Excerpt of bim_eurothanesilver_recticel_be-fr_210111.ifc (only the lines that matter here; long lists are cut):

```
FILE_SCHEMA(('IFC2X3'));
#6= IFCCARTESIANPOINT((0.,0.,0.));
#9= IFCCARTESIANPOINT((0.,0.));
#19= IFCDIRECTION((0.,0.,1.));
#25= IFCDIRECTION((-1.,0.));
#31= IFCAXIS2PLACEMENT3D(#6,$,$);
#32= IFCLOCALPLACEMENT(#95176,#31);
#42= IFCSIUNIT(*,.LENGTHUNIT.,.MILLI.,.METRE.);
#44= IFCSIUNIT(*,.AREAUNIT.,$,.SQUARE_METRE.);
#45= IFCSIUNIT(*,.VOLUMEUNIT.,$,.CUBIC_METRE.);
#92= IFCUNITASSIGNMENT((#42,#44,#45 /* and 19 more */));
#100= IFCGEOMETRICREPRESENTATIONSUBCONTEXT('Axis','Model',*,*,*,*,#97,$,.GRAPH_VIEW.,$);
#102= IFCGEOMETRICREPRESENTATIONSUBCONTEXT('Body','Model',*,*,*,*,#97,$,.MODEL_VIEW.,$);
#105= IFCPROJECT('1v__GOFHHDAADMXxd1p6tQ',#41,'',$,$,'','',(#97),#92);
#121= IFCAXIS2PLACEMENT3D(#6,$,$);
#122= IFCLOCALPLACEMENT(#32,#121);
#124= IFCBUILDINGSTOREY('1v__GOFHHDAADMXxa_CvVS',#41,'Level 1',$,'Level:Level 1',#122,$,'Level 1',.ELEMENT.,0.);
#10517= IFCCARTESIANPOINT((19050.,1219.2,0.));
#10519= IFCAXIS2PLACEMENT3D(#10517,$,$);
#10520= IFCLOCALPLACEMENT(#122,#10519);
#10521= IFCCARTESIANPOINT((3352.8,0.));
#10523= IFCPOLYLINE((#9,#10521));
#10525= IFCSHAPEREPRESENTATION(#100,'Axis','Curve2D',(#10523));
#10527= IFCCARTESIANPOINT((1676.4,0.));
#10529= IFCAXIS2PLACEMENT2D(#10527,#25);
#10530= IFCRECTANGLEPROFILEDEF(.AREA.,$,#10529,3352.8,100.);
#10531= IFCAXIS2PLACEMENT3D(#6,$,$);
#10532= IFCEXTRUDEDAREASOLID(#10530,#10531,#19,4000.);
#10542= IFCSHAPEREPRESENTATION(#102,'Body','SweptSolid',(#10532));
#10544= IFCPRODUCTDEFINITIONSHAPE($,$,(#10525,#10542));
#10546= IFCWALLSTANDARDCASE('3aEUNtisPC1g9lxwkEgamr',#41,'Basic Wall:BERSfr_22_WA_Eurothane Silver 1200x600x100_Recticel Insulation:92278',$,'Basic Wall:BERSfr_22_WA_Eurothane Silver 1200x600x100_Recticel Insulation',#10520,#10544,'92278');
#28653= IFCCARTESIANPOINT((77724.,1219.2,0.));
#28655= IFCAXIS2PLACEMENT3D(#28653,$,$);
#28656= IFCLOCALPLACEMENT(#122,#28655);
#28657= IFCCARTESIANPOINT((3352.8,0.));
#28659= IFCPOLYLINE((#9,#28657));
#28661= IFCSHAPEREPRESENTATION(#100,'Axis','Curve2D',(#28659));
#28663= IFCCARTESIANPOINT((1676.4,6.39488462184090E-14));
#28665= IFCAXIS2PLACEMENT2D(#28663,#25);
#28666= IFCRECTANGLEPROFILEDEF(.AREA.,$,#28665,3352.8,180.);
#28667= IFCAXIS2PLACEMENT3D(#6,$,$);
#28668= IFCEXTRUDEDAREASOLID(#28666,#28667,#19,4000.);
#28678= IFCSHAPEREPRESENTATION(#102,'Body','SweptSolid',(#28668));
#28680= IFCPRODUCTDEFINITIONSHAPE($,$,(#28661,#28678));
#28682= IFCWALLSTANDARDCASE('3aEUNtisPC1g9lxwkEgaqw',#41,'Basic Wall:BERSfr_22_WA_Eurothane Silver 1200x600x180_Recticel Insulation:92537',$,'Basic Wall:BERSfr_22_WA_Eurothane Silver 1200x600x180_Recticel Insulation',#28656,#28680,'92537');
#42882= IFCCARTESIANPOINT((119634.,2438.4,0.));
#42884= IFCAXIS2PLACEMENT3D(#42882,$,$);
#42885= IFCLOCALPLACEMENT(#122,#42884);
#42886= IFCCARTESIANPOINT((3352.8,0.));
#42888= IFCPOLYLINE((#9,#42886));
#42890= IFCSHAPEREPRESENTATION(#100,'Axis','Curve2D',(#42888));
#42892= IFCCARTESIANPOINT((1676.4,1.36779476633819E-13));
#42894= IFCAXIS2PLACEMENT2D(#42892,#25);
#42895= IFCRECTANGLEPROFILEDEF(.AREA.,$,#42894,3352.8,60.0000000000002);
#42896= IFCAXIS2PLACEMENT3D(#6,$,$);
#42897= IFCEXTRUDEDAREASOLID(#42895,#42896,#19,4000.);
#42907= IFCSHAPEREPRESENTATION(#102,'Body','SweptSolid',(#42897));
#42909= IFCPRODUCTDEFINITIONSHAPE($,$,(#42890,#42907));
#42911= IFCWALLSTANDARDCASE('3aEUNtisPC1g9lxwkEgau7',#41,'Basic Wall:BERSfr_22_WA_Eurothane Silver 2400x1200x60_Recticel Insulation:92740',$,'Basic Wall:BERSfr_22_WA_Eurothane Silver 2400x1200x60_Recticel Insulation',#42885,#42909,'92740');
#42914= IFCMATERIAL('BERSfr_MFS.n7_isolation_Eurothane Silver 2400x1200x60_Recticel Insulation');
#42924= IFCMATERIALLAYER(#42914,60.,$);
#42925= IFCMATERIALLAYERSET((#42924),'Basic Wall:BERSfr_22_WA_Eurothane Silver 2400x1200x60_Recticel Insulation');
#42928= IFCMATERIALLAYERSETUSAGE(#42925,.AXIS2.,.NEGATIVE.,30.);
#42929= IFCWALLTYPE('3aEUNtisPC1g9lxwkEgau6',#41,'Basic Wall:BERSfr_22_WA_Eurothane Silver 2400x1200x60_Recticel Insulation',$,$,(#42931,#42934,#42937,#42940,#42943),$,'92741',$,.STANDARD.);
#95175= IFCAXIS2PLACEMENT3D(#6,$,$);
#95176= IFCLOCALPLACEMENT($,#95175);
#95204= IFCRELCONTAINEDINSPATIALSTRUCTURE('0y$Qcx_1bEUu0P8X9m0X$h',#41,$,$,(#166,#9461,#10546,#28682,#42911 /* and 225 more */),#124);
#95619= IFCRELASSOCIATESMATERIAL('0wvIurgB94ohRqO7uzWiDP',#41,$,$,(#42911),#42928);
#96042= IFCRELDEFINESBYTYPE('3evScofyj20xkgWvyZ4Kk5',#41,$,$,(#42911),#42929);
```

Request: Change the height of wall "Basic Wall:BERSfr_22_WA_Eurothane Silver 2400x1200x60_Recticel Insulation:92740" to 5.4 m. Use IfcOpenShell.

```python
import ifcopenshell
import ifcopenshell.geom
import ifcopenshell.util.representation
import ifcopenshell.util.shape
import ifcopenshell.util.unit

model = ifcopenshell.open("bim_eurothanesilver_recticel_be-fr_210111.ifc")
unit_scale = ifcopenshell.util.unit.calculate_unit_scale(model)
settings = ifcopenshell.geom.settings()


def volume(element):
    """Net volume in cubic metres, openings subtracted."""
    shape = ifcopenshell.geom.create_shape(settings, element)
    return ifcopenshell.util.shape.get_volume(shape.geometry)


wall = model.by_guid("3aEUNtisPC1g9lxwkEgau7")
before = volume(wall)

body = ifcopenshell.util.representation.get_representation(wall, "Model", "Body")
solid = body.Items[0]
old_height = solid.Depth
solid.Depth = 5.4 / unit_scale
after = volume(wall)

print(f"height {old_height:g} -> {solid.Depth:g}, volume {before:.3f} -> {after:.3f} m3")

model.write("bim_eurothanesilver_recticel_be-fr_210111_rev.ifc")
```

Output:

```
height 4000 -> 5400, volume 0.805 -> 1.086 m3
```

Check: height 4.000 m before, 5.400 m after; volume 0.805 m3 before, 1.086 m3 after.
